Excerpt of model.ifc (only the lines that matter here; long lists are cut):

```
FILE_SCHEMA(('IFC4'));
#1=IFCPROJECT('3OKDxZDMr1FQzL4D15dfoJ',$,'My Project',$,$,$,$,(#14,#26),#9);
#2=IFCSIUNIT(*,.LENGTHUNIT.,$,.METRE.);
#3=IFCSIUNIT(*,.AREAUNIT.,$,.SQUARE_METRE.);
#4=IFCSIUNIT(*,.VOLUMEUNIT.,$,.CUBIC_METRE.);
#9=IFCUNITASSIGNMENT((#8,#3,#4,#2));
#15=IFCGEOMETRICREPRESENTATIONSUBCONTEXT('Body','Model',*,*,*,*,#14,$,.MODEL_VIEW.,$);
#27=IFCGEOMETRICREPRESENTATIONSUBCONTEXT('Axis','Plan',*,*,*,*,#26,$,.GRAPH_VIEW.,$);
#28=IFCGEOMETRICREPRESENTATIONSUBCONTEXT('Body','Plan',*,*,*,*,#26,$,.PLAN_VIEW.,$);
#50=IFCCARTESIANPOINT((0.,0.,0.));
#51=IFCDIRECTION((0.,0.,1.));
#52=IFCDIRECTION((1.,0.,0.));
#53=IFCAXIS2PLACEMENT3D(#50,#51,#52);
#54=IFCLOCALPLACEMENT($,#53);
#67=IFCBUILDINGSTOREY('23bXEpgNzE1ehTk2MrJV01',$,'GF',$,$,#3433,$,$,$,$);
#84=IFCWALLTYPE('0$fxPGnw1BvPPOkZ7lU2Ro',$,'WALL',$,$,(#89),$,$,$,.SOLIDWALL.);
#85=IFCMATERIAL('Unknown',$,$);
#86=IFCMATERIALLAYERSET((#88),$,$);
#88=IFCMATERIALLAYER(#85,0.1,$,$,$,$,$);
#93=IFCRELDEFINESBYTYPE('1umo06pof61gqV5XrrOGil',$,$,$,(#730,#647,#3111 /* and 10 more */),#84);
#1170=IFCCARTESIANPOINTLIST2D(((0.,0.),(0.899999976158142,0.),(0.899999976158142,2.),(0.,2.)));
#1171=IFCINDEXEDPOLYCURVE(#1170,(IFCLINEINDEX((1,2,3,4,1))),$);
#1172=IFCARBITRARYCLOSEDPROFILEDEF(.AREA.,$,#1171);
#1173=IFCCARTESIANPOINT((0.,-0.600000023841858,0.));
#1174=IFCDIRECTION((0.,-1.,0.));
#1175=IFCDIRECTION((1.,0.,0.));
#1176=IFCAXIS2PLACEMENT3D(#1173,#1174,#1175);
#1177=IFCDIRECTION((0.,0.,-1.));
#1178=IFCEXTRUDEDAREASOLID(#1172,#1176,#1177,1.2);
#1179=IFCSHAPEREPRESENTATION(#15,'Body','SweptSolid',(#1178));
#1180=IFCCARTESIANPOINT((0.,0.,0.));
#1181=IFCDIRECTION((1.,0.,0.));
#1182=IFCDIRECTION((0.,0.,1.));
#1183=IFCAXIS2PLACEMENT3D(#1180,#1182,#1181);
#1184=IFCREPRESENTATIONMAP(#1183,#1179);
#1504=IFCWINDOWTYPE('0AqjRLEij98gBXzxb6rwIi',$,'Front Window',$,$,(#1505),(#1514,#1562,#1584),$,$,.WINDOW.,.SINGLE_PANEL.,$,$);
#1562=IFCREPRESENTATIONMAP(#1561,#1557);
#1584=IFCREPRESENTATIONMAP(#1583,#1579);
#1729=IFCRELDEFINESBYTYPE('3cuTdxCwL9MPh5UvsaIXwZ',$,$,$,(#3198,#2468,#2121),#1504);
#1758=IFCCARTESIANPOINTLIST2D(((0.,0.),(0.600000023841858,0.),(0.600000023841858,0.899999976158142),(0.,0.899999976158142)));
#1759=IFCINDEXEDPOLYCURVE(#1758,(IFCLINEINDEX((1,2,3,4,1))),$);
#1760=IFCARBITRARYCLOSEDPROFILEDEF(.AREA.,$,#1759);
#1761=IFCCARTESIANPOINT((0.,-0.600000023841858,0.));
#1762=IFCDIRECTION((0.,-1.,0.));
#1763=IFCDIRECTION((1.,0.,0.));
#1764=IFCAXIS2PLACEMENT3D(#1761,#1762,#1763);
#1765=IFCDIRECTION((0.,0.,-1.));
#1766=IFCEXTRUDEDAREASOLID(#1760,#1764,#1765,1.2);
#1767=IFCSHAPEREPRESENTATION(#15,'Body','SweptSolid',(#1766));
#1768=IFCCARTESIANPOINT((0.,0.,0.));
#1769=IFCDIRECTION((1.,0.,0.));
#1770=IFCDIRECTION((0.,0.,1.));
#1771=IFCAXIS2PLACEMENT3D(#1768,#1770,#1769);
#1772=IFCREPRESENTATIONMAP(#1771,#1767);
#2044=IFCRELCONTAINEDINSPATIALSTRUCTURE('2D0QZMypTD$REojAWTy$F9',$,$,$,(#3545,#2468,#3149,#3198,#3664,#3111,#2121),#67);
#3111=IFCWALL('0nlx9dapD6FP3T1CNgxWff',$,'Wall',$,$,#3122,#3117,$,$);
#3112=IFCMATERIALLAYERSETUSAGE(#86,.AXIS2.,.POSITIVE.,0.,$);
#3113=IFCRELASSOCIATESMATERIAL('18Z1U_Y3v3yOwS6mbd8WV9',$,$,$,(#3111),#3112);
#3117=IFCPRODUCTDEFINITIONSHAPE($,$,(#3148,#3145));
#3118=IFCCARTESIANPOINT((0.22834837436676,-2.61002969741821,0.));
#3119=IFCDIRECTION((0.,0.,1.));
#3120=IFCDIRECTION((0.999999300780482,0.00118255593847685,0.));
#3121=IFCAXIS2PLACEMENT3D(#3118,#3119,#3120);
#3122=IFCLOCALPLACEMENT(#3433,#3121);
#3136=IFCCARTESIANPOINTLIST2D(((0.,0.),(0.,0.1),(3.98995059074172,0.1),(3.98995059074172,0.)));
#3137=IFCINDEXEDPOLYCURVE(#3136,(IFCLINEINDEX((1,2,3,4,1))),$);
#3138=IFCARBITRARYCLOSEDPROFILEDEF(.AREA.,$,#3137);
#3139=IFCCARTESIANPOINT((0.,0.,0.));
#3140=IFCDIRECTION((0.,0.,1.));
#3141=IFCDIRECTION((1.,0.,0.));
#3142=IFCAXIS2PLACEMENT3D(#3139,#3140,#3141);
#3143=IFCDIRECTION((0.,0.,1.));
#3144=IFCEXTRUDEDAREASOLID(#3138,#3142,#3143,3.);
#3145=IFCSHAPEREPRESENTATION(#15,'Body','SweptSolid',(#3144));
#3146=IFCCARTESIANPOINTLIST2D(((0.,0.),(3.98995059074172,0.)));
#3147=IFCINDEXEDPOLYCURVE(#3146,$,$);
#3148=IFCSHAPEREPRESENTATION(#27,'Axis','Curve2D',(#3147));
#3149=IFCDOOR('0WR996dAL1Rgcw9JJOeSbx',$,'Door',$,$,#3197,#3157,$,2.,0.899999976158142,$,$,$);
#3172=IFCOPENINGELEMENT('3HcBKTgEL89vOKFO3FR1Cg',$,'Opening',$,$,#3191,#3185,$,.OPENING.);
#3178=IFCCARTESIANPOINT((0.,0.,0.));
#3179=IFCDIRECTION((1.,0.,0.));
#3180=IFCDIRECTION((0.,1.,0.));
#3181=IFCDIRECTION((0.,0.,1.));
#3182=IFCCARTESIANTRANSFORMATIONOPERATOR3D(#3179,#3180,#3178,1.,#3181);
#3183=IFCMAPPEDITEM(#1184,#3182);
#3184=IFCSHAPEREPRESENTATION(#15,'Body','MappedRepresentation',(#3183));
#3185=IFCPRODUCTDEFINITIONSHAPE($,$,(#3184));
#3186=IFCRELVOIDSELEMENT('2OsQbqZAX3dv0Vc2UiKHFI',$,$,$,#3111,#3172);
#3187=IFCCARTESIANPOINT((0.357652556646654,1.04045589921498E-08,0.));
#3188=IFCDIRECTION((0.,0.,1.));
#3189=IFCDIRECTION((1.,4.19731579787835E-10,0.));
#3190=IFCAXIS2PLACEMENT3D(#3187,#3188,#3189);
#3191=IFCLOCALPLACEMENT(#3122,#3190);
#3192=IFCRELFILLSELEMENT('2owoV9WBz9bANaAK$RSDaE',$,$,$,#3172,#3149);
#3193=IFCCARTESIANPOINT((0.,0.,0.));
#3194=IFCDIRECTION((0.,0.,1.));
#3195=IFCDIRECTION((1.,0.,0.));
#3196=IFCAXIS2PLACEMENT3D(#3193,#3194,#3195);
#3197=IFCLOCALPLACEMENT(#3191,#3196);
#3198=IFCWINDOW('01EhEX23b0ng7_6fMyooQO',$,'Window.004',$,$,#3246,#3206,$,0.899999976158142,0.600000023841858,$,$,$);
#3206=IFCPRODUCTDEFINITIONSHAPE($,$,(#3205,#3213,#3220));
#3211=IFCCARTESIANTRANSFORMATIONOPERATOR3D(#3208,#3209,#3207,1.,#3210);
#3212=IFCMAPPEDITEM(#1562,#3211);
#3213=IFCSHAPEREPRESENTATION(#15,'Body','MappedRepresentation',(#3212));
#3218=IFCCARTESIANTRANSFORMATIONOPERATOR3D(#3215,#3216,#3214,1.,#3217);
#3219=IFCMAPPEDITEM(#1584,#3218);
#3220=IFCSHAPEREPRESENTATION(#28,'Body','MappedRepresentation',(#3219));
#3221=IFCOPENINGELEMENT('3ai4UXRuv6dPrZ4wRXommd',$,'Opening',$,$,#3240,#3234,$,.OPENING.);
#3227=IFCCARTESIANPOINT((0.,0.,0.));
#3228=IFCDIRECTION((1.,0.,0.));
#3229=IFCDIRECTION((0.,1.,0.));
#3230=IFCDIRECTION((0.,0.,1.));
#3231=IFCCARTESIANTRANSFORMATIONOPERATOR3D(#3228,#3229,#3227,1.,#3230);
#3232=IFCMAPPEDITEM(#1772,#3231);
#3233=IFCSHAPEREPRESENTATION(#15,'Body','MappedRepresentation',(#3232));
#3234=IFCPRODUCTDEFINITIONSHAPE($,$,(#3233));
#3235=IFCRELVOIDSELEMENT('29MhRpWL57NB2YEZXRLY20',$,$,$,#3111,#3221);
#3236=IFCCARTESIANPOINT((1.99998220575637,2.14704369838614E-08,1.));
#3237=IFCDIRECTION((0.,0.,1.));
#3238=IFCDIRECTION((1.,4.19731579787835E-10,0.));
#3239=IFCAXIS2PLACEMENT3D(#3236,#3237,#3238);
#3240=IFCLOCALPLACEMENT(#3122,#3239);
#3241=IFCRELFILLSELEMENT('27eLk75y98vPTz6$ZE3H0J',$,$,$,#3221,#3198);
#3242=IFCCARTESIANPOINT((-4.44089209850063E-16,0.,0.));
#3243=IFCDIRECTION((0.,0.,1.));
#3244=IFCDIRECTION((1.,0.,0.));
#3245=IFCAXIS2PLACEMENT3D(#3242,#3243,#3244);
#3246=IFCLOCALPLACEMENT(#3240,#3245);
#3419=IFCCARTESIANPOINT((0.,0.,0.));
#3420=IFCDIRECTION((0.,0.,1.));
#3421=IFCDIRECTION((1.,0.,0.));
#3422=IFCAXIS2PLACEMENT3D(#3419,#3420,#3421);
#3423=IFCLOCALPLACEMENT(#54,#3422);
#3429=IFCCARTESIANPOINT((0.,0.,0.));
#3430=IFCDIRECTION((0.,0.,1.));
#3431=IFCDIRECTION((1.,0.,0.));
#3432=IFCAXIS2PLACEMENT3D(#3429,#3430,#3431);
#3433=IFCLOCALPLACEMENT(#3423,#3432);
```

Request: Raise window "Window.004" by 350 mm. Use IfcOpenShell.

```python
import numpy as np
import ifcopenshell
import ifcopenshell.api.geometry
import ifcopenshell.util.placement
import ifcopenshell.util.unit

model = ifcopenshell.open("model.ifc")
unit_scale = ifcopenshell.util.unit.calculate_unit_scale(model)

window = model.by_id(3198)
opening = window.FillsVoids[0].RelatingOpeningElement
dz = 0.35 / unit_scale

shift = np.array([0.0, 0.0, dz])
# The window is placed relative to its opening, so it follows when the opening moves.
matrix = ifcopenshell.util.placement.get_local_placement(opening.ObjectPlacement)
matrix[:3, 3] += shift
ifcopenshell.api.geometry.edit_object_placement(
    model, product=opening, matrix=matrix, is_si=False, should_transform_children=True
)

print(f"moved by {dz * unit_scale:+.3f} m")

model.write("model_updated.ifc")
```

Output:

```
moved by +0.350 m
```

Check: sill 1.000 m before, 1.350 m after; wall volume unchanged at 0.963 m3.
